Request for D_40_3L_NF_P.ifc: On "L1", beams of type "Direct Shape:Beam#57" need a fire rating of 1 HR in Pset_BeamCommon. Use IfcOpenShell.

First a look at what the model holds.

```python
import ifcopenshell
import ifcopenshell.util.element

model = ifcopenshell.open("D_40_3L_NF_P.ifc")
print(model.schema)
storey = next(s for s in model.by_type("IfcBuildingStorey") if s.Name == "L1")
beams = [e for e in ifcopenshell.util.element.get_decomposition(storey) if e.is_a("IfcBeam")]
seen = {}
for e in beams:
    element_type = ifcopenshell.util.element.get_type(e)
    key = (element_type.Name if element_type != e and element_type else None, ifcopenshell.util.element.get_pset(e, "Pset_BeamCommon", "FireRating"))
    seen[key] = seen.get(key, 0) + 1
for (name, value), count in sorted(seen.items(), key=str):
    print(count, "x", name, "|", value)
```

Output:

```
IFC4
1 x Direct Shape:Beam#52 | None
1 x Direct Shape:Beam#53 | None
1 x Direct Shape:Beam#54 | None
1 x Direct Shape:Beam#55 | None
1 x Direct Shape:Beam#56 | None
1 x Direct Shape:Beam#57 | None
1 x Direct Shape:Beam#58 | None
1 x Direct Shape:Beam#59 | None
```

```python
import ifcopenshell
import ifcopenshell.api.pset
import ifcopenshell.util.element

model = ifcopenshell.open("D_40_3L_NF_P.ifc")

storey = next(s for s in model.by_type("IfcBuildingStorey") if s.Name == "L1")
beams = [e for e in ifcopenshell.util.element.get_decomposition(storey) if e.is_a("IfcBeam")]

count = 0
for e in beams:
    element_type = ifcopenshell.util.element.get_type(e)
    if element_type in (None, e) or element_type.Name != "Direct Shape:Beam#57":
        continue
    # add_pset returns the element's existing set when there is one.
    pset = ifcopenshell.api.pset.add_pset(model, product=e, name="Pset_BeamCommon")
    ifcopenshell.api.pset.edit_pset(model, pset=pset, properties={"FireRating": "1 HR"})
    count += 1

print(count, "beams updated")

model.write("D_40_3L_NF_P_updated.ifc")
```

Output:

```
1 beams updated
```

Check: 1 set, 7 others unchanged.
